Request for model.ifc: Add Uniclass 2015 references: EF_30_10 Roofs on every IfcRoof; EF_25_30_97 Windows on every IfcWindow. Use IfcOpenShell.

First a look at what the model holds.

```python
import ifcopenshell

model = ifcopenshell.open("model.ifc")
print(model.schema)
print("classifications:", [c.Name for c in model.by_type("IfcClassification")])
for ifc_class in ("IfcDoor", "IfcRoof", "IfcStair", "IfcWall", "IfcWindow"):
    print(ifc_class, len(model.by_type(ifc_class)))
```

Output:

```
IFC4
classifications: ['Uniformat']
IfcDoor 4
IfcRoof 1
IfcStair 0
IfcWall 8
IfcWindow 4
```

```python
import ifcopenshell
import ifcopenshell.api.classification

model = ifcopenshell.open("model.ifc")

system = ifcopenshell.api.classification.add_classification(model, classification="Uniclass 2015")

codes = {
    "IfcRoof": ("EF_30_10", "Roofs"),
    "IfcWindow": ("EF_25_30_97", "Windows"),
}
for ifc_class, (code, name) in codes.items():
    products = model.by_type(ifc_class)
    ifcopenshell.api.classification.add_reference(
        model, products=products, classification=system, identification=code, name=name
    )
    print(code, len(products))

model.write("model_v2.ifc")
```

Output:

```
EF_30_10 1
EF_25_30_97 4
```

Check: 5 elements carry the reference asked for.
